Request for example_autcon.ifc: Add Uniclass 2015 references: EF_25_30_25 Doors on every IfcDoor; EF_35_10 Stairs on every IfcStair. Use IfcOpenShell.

First a look at what the model holds.

```python
import ifcopenshell

model = ifcopenshell.open("example_autcon.ifc")
print(model.schema)
print("classifications:", [c.Name for c in model.by_type("IfcClassification")])
for ifc_class in ("IfcDoor", "IfcRoof", "IfcStair", "IfcWall", "IfcWindow"):
    print(ifc_class, len(model.by_type(ifc_class)))
```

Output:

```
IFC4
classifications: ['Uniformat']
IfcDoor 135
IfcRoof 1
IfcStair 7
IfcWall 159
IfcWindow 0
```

```python
import ifcopenshell
import ifcopenshell.api.classification

model = ifcopenshell.open("example_autcon.ifc")

system = ifcopenshell.api.classification.add_classification(model, classification="Uniclass 2015")

codes = {
    "IfcDoor": ("EF_25_30_25", "Doors"),
    "IfcStair": ("EF_35_10", "Stairs"),
}
for ifc_class, (code, name) in codes.items():
    products = model.by_type(ifc_class)
    ifcopenshell.api.classification.add_reference(
        model, products=products, classification=system, identification=code, name=name
    )
    print(code, len(products))

model.write("example_autcon_edited.ifc")
```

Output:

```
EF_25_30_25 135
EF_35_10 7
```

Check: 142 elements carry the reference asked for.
